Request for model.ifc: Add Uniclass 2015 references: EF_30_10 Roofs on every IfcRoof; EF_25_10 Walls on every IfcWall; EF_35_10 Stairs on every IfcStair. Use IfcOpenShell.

First a look at what the model holds.

```python
import ifcopenshell

model = ifcopenshell.open("model.ifc")
print(model.schema)
print("classifications:", [c.Name for c in model.by_type("IfcClassification")])
for ifc_class in ("IfcDoor", "IfcRoof", "IfcStair", "IfcWall", "IfcWindow"):
    print(ifc_class, len(model.by_type(ifc_class)))
```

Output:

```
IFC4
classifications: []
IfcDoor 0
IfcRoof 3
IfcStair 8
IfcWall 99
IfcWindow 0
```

```python
import ifcopenshell
import ifcopenshell.api.classification

model = ifcopenshell.open("model.ifc")

system = ifcopenshell.api.classification.add_classification(model, classification="Uniclass 2015")

codes = {
    "IfcRoof": ("EF_30_10", "Roofs"),
    "IfcWall": ("EF_25_10", "Walls"),
    "IfcStair": ("EF_35_10", "Stairs"),
}
for ifc_class, (code, name) in codes.items():
    products = model.by_type(ifc_class)
    ifcopenshell.api.classification.add_reference(
        model, products=products, classification=system, identification=code, name=name
    )
    print(code, len(products))

model.write("model_updated.ifc")
```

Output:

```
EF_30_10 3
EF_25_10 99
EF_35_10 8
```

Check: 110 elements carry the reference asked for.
